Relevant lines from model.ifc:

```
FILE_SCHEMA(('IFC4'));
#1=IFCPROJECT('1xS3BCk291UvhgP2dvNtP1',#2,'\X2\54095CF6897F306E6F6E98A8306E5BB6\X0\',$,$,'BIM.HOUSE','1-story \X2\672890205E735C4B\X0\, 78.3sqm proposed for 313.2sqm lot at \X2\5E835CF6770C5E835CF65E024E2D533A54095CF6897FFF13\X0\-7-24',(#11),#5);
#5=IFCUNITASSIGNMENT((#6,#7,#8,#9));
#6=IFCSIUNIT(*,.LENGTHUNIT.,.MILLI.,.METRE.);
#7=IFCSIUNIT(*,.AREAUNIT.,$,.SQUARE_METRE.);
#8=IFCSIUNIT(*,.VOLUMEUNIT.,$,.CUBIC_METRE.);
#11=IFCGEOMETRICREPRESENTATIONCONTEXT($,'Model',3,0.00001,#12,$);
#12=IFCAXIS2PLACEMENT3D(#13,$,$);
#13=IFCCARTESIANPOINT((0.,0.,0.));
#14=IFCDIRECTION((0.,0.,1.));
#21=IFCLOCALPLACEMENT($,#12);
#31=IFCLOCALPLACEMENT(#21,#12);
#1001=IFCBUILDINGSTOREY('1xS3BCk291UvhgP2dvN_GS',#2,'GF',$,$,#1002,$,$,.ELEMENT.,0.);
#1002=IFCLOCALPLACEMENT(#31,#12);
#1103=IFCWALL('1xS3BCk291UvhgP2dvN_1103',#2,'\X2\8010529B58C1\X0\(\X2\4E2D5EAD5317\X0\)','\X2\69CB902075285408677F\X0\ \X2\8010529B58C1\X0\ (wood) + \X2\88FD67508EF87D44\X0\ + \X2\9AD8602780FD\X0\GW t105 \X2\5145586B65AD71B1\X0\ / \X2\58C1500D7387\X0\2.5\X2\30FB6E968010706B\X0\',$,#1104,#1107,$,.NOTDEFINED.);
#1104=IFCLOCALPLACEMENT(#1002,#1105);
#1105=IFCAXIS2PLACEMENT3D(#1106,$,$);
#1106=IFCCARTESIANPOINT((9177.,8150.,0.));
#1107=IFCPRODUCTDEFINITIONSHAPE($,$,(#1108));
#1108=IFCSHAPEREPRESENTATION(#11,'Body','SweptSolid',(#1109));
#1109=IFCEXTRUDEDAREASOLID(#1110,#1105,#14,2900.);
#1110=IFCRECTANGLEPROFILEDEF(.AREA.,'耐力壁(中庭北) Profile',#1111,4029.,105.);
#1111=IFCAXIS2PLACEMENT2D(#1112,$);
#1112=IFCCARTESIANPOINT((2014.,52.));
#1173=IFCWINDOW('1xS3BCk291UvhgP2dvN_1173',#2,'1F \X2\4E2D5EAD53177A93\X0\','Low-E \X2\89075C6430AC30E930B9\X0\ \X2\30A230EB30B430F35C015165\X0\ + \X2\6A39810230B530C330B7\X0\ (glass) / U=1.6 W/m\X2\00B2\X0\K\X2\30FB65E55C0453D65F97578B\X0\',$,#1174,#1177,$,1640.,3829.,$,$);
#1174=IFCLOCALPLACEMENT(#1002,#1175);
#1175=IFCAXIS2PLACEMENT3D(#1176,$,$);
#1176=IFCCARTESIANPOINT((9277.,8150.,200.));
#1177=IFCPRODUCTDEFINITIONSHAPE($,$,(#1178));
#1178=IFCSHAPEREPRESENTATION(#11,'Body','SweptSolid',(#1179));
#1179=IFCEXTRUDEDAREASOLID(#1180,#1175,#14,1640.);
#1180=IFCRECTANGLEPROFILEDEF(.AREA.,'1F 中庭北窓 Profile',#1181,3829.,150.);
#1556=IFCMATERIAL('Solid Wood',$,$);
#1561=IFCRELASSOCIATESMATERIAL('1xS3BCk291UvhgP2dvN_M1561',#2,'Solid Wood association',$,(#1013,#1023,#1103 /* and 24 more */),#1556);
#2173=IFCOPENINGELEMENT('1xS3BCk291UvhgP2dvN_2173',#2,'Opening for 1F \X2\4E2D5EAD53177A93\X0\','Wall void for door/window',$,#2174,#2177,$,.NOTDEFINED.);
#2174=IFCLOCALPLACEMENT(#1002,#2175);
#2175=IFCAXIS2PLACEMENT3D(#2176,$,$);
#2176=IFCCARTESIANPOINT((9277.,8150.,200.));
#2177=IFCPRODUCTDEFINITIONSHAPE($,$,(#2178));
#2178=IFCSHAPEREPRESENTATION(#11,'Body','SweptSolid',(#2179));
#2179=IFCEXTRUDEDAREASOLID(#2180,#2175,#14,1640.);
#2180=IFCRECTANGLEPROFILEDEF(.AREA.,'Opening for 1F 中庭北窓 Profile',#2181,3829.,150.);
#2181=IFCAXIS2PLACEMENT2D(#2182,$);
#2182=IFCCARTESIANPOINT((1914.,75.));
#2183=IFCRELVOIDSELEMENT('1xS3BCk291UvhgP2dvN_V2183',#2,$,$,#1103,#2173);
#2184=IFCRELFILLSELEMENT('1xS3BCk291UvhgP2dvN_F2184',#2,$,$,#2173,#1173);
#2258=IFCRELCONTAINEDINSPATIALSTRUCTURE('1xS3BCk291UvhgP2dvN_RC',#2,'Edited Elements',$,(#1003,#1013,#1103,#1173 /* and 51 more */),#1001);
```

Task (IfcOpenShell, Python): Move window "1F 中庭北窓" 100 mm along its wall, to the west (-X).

```python
import ifcopenshell
import ifcopenshell.api.geometry
import ifcopenshell.util.placement
import ifcopenshell.util.unit

model = ifcopenshell.open("model.ifc")
unit_scale = ifcopenshell.util.unit.calculate_unit_scale(model)

window = model.by_guid("1xS3BCk291UvhgP2dvN_1173")
opening = window.FillsVoids[0].RelatingOpeningElement
wall = opening.VoidsElements[0].RelatingBuildingElement

wall_matrix = ifcopenshell.util.placement.get_local_placement(wall.ObjectPlacement)
shift = wall_matrix[:3, 0] * -0.1 / unit_scale
before = ifcopenshell.util.placement.get_local_placement(window.ObjectPlacement)[:3, 3].copy()

# The window is not placed relative to its opening, so move both.
for product in (opening, window):
    matrix = ifcopenshell.util.placement.get_local_placement(product.ObjectPlacement)
    matrix[:3, 3] += shift
    ifcopenshell.api.geometry.edit_object_placement(model, product=product, matrix=matrix, is_si=False)

after = ifcopenshell.util.placement.get_local_placement(window.ObjectPlacement)[:3, 3]
print("window moved by", (after - before).round(3) + 0.0)

model.write("model_v2.ifc")
```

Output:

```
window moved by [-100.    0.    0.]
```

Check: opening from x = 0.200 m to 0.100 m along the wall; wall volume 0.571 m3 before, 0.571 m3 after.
